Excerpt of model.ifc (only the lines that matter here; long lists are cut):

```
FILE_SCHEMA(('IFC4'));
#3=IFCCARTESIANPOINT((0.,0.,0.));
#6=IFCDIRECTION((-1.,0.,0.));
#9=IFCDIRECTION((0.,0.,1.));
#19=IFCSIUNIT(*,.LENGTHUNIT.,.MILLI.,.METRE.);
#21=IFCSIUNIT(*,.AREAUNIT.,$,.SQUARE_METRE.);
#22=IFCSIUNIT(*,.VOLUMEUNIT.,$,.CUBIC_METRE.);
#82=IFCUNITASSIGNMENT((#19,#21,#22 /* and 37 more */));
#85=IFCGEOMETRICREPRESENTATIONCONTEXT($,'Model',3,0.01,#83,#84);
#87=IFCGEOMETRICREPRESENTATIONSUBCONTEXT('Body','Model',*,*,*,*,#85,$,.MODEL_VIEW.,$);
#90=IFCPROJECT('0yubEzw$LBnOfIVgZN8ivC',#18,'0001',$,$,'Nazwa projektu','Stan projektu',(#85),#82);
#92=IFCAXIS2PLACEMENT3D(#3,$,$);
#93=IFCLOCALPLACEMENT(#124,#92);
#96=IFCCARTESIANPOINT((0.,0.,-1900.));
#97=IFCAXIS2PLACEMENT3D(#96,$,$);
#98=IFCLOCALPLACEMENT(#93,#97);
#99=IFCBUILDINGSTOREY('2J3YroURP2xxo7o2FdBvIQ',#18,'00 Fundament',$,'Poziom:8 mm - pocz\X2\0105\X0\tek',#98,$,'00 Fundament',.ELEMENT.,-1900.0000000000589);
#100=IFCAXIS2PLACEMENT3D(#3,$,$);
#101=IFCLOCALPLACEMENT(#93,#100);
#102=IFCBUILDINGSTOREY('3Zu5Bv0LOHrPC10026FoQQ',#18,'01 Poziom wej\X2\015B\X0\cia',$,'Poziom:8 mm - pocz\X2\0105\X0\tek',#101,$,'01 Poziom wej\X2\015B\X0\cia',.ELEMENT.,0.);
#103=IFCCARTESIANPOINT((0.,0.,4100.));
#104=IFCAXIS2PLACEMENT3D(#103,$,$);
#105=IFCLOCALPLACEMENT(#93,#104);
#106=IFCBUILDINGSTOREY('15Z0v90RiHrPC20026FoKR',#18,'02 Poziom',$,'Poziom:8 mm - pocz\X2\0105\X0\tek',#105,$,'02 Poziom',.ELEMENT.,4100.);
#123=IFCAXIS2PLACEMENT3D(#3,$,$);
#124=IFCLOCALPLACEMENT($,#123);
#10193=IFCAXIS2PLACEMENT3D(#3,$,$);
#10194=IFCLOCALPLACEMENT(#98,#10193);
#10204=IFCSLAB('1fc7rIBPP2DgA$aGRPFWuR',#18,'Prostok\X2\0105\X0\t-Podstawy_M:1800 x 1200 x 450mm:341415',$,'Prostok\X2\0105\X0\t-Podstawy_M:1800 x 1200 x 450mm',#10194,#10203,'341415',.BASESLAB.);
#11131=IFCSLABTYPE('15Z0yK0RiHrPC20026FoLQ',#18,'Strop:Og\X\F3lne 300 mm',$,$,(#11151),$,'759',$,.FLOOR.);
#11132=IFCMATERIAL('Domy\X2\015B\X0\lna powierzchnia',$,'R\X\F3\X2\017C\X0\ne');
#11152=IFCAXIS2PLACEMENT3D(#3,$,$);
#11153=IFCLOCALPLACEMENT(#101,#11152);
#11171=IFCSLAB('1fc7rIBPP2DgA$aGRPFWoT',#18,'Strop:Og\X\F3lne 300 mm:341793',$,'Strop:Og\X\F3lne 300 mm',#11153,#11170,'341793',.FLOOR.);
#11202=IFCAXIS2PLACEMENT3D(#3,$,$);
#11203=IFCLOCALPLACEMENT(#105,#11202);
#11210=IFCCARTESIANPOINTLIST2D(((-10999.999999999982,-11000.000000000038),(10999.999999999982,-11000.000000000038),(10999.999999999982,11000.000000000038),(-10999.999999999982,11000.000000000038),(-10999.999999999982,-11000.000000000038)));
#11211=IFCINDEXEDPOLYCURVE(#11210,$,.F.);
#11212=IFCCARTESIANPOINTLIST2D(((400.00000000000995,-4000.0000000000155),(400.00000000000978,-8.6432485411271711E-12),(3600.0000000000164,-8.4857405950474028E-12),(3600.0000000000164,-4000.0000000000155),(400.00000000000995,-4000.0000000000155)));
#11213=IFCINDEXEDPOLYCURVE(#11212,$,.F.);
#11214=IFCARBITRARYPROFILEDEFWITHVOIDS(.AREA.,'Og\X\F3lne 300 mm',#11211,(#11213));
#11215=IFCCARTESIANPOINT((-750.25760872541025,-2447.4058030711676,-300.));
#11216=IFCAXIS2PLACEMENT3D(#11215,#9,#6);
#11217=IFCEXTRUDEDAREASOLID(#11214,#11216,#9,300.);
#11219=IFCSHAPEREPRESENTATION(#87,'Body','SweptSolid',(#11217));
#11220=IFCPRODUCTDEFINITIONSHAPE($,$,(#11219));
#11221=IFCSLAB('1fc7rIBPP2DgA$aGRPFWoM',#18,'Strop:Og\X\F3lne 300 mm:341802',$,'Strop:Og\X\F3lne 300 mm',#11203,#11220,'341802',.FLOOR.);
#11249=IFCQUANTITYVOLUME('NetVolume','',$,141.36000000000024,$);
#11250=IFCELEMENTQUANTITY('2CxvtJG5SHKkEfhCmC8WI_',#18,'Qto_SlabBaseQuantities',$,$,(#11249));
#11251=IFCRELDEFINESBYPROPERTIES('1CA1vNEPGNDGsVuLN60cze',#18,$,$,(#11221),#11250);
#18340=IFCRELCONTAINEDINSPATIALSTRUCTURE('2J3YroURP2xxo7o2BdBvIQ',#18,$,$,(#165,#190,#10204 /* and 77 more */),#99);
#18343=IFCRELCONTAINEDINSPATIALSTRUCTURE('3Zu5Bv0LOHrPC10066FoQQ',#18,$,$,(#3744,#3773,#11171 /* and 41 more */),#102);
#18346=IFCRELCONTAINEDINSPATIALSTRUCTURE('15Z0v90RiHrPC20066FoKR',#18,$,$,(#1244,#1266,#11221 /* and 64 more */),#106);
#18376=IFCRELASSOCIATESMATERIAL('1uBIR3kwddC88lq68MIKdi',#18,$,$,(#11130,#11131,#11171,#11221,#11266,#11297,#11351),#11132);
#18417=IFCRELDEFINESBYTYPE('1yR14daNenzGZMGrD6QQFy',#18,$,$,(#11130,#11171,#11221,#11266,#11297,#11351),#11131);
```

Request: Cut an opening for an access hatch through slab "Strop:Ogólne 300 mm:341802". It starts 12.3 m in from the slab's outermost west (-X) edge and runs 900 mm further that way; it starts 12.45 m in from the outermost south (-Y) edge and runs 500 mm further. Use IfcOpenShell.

```python
import numpy as np
import ifcopenshell
import ifcopenshell.api.feature
import ifcopenshell.api.geometry
import ifcopenshell.api.pset
import ifcopenshell.api.root
import ifcopenshell.geom
import ifcopenshell.util.element
import ifcopenshell.util.placement
import ifcopenshell.util.representation
import ifcopenshell.util.shape
import ifcopenshell.util.unit

model = ifcopenshell.open("model.ifc")
unit_scale = ifcopenshell.util.unit.calculate_unit_scale(model)
volume_scale = ifcopenshell.util.unit.calculate_unit_scale(model, "VOLUMEUNIT")
settings = ifcopenshell.geom.settings()


def volume(element):
    """Net volume in cubic metres, openings subtracted."""
    shape = ifcopenshell.geom.create_shape(settings, element)
    return ifcopenshell.util.shape.get_volume(shape.geometry)


slab = model.by_id(11221)
before = volume(slab)

# Extent in the slab's own axes, in metres. The edges named are its -X and -Y sides.
slab_shape = ifcopenshell.geom.create_shape(settings, slab)
vertices = ifcopenshell.util.shape.get_vertices(slab_shape.geometry)
x_min, y_min, bottom = vertices.min(axis=0)
top = vertices[:, 2].max()

opening = ifcopenshell.api.root.create_entity(model, ifc_class="IfcOpeningElement", name="Access hatch opening", predefined_type="OPENING")
context = ifcopenshell.util.representation.get_context(model, "Model", "Body", "MODEL_VIEW")
width, depth = 0.9, 0.5
outline = [(0.0, 0.0), (width, 0.0), (width, depth), (0.0, depth), (0.0, 0.0)]
# Overshoot both faces by 50 mm so the cut is clean.
shape = ifcopenshell.api.geometry.add_slab_representation(
    model, context=context, depth=top - bottom + 0.1, polyline=outline
)
ifcopenshell.api.geometry.assign_representation(model, product=opening, representation=shape)

matrix = ifcopenshell.util.placement.get_local_placement(slab.ObjectPlacement)
matrix[:, 3] = matrix @ np.append(np.array([x_min + 12.3, y_min + 12.45, bottom - 0.05]) / unit_scale, 1.0)
ifcopenshell.api.geometry.edit_object_placement(model, product=opening, matrix=matrix, is_si=False)
ifcopenshell.api.feature.add_feature(model, feature=opening, element=slab)

after = volume(slab)

# Update the slab's stored quantities.
qto = model.by_id(ifcopenshell.util.element.get_pset(slab, "Qto_SlabBaseQuantities", should_inherit=False)["id"])
ifcopenshell.api.pset.edit_qto(model, qto=qto, properties={"NetVolume": after / volume_scale})

print(f"slab volume {before:.3f} -> {after:.3f} m3")

model.write("model_edited.ifc")
```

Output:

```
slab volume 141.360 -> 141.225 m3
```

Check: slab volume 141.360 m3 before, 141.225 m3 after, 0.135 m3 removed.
